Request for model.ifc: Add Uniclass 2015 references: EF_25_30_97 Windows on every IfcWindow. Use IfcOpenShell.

First a look at what the model holds.

```python
import ifcopenshell

model = ifcopenshell.open("model.ifc")
print(model.schema)
print("classifications:", [c.Name for c in model.by_type("IfcClassification")])
for ifc_class in ("IfcDoor", "IfcRoof", "IfcStair", "IfcWall", "IfcWindow"):
    print(ifc_class, len(model.by_type(ifc_class)))
```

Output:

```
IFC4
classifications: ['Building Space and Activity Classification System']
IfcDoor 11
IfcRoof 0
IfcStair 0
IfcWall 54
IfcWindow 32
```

```python
import ifcopenshell
import ifcopenshell.api.classification

model = ifcopenshell.open("model.ifc")

system = ifcopenshell.api.classification.add_classification(model, classification="Uniclass 2015")

codes = {
    "IfcWindow": ("EF_25_30_97", "Windows"),
}
for ifc_class, (code, name) in codes.items():
    products = model.by_type(ifc_class)
    ifcopenshell.api.classification.add_reference(
        model, products=products, classification=system, identification=code, name=name
    )
    print(code, len(products))

model.write("model_rev.ifc")
```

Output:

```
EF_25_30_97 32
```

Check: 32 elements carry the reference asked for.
